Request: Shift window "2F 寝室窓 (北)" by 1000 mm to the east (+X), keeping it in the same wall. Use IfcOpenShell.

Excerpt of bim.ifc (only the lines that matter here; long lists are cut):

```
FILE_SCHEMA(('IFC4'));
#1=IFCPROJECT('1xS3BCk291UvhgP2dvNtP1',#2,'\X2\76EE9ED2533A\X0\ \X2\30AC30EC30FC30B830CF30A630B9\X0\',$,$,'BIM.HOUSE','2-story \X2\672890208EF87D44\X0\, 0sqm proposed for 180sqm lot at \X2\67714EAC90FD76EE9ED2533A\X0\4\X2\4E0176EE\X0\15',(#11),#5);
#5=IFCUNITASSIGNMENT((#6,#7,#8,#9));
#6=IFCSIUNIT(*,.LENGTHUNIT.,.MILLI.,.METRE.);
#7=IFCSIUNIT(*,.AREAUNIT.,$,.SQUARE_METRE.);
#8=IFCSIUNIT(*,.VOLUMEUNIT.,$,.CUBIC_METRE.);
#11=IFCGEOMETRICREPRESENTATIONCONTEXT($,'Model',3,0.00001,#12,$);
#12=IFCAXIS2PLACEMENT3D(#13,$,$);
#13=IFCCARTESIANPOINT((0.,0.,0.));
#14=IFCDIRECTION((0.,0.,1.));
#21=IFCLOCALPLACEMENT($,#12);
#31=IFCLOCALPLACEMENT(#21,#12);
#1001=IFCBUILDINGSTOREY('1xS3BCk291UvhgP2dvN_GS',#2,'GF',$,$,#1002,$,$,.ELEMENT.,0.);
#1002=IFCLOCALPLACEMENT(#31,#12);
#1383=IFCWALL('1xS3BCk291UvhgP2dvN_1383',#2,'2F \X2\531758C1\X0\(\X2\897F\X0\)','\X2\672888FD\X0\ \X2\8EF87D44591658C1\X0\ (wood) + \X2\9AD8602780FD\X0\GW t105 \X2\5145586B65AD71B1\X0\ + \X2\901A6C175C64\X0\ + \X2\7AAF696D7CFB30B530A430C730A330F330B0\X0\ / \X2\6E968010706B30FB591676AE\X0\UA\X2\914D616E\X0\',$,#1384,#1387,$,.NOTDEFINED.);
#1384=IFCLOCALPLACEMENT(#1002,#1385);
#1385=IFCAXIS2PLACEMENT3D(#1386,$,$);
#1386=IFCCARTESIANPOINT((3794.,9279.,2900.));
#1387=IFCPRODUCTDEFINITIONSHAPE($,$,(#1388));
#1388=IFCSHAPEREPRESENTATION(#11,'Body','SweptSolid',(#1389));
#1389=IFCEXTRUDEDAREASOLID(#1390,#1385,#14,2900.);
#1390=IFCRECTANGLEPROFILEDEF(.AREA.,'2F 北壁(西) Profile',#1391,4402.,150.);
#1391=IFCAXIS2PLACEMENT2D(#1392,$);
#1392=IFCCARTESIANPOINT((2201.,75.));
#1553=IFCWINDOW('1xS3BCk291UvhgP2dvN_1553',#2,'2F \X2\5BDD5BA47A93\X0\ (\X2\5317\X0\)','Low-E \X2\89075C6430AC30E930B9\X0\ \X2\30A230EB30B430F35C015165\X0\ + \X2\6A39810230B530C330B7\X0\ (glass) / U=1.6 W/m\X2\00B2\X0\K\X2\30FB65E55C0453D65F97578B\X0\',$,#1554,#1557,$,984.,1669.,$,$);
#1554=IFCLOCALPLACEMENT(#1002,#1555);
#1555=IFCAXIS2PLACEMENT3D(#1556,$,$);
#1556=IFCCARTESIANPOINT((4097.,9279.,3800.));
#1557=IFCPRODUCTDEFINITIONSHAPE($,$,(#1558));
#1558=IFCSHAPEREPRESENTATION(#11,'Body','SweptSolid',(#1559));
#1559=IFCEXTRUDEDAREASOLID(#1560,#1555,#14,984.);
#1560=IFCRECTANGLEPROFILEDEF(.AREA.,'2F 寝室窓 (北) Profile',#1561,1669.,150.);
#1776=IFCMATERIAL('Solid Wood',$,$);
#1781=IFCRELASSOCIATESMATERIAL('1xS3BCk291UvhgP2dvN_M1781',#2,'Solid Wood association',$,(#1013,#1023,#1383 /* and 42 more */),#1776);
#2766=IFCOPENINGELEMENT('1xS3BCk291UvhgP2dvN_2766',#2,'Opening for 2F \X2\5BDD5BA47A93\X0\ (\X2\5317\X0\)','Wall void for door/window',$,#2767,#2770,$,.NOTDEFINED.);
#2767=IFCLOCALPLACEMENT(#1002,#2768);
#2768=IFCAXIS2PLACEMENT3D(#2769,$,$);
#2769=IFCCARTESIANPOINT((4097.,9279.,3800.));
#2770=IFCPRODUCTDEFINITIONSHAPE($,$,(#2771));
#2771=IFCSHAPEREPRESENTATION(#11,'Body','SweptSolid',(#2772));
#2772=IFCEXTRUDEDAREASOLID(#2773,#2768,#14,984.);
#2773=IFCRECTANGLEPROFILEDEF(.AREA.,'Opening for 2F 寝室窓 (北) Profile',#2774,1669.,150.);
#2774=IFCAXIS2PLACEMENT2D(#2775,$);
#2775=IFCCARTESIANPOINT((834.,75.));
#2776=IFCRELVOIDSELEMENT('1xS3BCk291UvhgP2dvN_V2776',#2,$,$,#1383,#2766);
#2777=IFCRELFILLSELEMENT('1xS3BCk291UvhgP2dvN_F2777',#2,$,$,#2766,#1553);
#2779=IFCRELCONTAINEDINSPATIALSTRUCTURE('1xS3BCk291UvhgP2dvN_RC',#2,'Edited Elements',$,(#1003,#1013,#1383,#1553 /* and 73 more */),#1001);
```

```python
import ifcopenshell
import ifcopenshell.api.geometry
import ifcopenshell.util.placement

model = ifcopenshell.open("bim.ifc")

window = model.by_guid("1xS3BCk291UvhgP2dvN_1553")
opening = window.FillsVoids[0].RelatingOpeningElement
wall = opening.VoidsElements[0].RelatingBuildingElement

wall_matrix = ifcopenshell.util.placement.get_local_placement(wall.ObjectPlacement)
shift = wall_matrix[:3, 0] * 1000.0
before = ifcopenshell.util.placement.get_local_placement(window.ObjectPlacement)[:3, 3].copy()

# The window is not placed relative to its opening, so move both.
for product in (opening, window):
    matrix = ifcopenshell.util.placement.get_local_placement(product.ObjectPlacement)
    matrix[:3, 3] += shift
    ifcopenshell.api.geometry.edit_object_placement(model, product=product, matrix=matrix, is_si=False)

after = ifcopenshell.util.placement.get_local_placement(window.ObjectPlacement)[:3, 3]
print("window moved by", (after - before).round(3) + 0.0)

model.write("bim_edited.ifc")
```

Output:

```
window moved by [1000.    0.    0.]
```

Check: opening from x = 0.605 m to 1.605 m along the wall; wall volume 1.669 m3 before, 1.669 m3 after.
